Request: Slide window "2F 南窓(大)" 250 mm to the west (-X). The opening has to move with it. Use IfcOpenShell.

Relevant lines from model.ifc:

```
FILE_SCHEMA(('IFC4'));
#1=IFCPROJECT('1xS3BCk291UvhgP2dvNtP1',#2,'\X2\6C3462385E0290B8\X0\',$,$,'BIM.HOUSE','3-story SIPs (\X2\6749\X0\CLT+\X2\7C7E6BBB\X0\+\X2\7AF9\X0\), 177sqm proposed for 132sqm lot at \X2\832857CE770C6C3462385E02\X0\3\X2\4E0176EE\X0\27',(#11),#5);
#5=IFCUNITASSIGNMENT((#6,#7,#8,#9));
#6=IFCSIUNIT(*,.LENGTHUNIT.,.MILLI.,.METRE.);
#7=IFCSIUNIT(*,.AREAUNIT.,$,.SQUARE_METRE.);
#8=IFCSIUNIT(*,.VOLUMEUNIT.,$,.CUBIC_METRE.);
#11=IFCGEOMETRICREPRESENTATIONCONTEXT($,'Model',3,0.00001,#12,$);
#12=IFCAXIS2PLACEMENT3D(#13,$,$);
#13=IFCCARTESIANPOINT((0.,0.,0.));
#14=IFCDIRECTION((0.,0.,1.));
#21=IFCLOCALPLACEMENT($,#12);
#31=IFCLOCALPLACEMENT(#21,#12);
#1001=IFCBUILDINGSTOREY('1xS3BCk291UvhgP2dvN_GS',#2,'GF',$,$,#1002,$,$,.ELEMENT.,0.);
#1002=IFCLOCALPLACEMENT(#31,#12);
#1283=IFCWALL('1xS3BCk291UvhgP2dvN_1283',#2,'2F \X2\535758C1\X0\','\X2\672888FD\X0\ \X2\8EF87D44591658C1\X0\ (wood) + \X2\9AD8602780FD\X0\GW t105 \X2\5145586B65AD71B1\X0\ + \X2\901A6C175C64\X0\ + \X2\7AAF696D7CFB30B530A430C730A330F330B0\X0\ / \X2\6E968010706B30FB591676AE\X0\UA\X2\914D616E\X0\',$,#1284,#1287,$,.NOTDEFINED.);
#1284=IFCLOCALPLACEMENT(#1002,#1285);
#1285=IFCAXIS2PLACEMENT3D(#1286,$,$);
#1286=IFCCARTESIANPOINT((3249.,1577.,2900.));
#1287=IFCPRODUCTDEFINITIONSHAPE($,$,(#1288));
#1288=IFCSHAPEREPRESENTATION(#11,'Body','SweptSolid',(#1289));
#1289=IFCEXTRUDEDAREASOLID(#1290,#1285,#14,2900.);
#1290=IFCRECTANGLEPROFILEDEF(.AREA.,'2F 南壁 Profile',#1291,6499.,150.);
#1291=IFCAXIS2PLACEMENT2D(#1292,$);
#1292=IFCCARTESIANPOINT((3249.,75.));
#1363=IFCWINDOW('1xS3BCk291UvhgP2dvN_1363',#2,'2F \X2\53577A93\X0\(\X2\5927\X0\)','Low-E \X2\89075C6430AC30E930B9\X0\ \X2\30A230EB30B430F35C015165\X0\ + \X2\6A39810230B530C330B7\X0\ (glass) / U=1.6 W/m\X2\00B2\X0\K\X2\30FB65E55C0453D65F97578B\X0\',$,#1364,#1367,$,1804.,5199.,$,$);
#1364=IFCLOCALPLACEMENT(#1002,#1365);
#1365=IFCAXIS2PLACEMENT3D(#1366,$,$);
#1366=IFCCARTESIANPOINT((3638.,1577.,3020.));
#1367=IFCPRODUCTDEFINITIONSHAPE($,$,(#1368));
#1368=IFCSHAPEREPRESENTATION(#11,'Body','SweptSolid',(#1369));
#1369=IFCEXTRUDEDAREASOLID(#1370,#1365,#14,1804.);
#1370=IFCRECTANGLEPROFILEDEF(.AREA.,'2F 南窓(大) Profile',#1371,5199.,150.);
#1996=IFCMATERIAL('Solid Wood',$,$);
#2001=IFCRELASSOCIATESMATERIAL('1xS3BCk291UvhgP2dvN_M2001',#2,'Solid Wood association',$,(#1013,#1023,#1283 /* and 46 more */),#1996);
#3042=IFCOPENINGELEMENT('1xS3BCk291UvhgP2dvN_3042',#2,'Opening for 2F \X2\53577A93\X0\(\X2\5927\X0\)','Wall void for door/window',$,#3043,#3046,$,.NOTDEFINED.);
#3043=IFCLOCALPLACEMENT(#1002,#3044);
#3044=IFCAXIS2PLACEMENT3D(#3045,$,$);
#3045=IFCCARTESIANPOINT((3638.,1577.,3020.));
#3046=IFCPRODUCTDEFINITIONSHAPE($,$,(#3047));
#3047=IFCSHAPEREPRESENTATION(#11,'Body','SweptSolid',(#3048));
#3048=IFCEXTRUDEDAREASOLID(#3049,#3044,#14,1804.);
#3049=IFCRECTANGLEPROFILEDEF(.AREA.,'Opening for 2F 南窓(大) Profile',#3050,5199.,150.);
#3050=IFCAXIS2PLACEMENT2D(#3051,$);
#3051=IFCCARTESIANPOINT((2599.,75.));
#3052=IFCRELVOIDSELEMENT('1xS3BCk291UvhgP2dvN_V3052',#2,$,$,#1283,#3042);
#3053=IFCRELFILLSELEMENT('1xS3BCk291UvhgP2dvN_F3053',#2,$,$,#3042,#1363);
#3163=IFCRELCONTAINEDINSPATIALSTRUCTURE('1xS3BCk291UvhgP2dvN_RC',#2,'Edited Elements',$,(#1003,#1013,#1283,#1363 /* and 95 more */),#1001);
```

```python
import ifcopenshell
import ifcopenshell.api.geometry
import ifcopenshell.util.placement

model = ifcopenshell.open("model.ifc")

window = model.by_guid("1xS3BCk291UvhgP2dvN_1363")
opening = window.FillsVoids[0].RelatingOpeningElement
wall = opening.VoidsElements[0].RelatingBuildingElement

wall_matrix = ifcopenshell.util.placement.get_local_placement(wall.ObjectPlacement)
shift = wall_matrix[:3, 0] * -250.0
before = ifcopenshell.util.placement.get_local_placement(window.ObjectPlacement)[:3, 3].copy()

# The window is not placed relative to its opening, so move both.
for product in (opening, window):
    matrix = ifcopenshell.util.placement.get_local_placement(product.ObjectPlacement)
    matrix[:3, 3] += shift
    ifcopenshell.api.geometry.edit_object_placement(model, product=product, matrix=matrix, is_si=False)

after = ifcopenshell.util.placement.get_local_placement(window.ObjectPlacement)[:3, 3]
print("window moved by", (after - before).round(3) + 0.0)

model.write("model_edited.ifc")
```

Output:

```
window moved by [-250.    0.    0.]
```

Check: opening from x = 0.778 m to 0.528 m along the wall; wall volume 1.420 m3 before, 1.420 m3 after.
